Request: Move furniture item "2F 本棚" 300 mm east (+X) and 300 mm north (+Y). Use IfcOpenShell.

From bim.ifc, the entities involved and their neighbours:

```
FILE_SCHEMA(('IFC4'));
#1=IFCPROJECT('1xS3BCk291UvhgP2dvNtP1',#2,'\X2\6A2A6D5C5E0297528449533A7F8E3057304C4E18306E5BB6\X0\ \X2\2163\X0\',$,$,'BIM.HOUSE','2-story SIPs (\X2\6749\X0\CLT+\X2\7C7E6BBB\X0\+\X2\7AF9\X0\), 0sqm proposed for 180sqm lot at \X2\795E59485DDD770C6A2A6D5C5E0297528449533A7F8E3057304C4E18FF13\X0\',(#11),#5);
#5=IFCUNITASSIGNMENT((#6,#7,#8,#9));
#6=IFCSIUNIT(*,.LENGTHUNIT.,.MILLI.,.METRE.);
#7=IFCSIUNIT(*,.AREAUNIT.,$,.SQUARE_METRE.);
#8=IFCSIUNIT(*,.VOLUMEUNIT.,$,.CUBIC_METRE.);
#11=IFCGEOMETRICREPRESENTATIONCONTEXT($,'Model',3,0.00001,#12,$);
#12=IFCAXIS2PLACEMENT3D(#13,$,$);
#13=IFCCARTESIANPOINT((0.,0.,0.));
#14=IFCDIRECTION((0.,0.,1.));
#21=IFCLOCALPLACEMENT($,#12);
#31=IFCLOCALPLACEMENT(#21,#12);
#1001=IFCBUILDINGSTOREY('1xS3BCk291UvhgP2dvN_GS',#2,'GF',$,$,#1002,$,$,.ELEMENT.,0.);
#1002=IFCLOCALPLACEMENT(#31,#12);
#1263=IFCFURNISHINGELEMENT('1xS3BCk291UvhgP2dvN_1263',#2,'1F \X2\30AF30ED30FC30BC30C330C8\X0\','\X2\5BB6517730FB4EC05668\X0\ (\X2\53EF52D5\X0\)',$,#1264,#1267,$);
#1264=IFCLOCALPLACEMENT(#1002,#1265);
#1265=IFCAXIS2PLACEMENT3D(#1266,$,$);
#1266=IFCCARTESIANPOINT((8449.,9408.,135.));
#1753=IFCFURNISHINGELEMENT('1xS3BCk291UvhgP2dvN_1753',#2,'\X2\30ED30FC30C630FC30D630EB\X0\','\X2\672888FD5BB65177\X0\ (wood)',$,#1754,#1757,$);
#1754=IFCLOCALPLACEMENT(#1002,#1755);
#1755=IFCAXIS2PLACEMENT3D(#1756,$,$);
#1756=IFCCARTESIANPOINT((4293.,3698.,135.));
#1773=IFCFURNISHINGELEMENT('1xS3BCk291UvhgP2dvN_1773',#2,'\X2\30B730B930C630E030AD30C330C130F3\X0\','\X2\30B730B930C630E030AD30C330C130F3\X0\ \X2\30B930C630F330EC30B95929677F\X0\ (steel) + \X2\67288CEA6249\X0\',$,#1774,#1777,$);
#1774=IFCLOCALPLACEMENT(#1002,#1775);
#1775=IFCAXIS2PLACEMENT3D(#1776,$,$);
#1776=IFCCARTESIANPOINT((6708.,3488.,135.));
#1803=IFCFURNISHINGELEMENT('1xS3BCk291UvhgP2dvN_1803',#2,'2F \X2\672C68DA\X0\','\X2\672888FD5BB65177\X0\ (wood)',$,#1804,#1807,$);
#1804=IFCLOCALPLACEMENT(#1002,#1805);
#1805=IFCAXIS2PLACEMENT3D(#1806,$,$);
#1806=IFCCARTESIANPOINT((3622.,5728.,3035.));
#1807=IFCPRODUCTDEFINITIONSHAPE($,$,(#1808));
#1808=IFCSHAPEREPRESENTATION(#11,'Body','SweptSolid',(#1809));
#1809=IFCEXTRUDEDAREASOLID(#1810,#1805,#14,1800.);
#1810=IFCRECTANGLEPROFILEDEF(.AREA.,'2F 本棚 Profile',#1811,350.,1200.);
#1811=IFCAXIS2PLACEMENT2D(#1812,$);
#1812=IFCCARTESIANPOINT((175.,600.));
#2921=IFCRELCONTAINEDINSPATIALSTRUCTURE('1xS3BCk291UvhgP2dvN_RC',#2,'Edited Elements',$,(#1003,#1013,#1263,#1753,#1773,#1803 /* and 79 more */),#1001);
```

```python
import ifcopenshell
import ifcopenshell.api.geometry
import ifcopenshell.util.placement
import ifcopenshell.util.unit

model = ifcopenshell.open("bim.ifc")
unit_scale = ifcopenshell.util.unit.calculate_unit_scale(model)

item = model.by_guid("1xS3BCk291UvhgP2dvN_1803")
matrix = ifcopenshell.util.placement.get_local_placement(item.ObjectPlacement)
matrix[0, 3] += 0.3 / unit_scale
matrix[1, 3] += 0.3 / unit_scale
ifcopenshell.api.geometry.edit_object_placement(model, product=item, matrix=matrix, is_si=False)

print(ifcopenshell.util.placement.get_local_placement(item.ObjectPlacement).round(3) + 0.0)

model.write("bim_edited.ifc")
```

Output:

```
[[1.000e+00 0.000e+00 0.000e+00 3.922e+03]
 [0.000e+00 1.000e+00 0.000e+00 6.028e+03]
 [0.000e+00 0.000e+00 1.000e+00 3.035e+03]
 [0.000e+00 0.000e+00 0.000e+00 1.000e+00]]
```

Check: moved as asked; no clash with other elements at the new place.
